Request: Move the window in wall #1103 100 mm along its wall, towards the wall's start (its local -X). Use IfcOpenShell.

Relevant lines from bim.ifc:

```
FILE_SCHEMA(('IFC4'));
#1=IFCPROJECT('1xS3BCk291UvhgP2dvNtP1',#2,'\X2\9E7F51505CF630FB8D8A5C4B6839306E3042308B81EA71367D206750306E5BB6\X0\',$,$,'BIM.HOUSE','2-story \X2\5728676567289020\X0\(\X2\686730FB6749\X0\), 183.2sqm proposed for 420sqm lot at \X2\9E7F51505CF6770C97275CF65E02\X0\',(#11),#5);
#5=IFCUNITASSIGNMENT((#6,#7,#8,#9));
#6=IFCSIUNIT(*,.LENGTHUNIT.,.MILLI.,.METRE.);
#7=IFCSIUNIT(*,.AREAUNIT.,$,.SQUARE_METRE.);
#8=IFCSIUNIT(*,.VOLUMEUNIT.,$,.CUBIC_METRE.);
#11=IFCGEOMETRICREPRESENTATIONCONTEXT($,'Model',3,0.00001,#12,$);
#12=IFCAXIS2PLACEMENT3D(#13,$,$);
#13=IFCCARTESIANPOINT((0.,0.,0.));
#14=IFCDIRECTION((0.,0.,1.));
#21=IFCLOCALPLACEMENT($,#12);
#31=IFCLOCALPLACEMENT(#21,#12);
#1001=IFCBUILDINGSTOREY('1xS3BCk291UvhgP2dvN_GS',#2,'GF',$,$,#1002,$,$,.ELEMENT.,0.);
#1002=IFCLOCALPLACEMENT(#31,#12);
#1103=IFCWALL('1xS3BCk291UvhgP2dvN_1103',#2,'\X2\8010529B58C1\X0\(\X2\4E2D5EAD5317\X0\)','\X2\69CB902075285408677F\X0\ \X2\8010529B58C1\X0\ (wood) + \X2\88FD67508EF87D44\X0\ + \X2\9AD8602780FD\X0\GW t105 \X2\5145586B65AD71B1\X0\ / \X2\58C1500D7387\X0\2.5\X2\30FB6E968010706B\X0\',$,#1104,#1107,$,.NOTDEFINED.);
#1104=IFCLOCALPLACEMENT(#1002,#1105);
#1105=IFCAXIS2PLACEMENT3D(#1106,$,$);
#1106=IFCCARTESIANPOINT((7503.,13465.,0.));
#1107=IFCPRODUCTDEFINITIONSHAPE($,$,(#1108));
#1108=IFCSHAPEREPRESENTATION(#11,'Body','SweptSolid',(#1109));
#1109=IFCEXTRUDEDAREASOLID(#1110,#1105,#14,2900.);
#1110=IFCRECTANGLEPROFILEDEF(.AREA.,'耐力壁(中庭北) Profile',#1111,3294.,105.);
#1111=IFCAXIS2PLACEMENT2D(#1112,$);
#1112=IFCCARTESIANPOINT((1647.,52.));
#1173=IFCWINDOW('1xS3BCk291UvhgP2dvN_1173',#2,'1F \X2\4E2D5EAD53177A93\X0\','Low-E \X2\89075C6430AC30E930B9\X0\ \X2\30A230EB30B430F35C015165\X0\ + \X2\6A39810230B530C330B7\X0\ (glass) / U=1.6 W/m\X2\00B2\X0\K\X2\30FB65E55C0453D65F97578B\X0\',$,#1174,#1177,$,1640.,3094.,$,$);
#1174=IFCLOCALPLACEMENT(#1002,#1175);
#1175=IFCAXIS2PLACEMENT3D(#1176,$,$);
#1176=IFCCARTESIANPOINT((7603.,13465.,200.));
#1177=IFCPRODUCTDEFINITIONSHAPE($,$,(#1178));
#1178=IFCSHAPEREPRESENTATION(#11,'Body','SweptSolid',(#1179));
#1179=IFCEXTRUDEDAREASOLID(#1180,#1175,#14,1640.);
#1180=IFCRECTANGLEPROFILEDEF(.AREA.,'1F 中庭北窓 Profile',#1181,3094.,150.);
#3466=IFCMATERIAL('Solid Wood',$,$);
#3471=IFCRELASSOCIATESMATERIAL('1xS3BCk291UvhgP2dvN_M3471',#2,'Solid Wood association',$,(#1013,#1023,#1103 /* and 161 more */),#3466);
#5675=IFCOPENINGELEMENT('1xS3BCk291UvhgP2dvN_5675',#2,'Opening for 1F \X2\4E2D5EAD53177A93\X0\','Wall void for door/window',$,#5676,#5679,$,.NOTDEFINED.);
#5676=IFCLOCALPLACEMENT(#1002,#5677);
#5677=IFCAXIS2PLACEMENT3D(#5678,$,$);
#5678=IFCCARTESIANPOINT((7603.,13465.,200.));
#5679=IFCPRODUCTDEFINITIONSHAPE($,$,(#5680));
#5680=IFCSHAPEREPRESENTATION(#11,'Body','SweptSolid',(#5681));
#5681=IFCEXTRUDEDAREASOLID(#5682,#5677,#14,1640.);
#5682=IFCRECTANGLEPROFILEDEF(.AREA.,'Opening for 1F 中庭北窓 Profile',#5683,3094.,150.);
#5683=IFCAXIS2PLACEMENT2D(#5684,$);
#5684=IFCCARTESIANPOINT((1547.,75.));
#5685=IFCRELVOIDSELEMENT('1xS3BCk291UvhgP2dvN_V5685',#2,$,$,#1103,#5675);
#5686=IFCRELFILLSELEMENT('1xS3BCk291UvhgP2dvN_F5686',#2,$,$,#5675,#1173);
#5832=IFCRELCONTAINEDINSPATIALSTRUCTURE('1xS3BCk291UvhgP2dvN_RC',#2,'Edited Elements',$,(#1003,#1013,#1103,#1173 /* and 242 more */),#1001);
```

```python
import ifcopenshell
import ifcopenshell.api.geometry
import ifcopenshell.util.placement
import ifcopenshell.util.unit

model = ifcopenshell.open("bim.ifc")
unit_scale = ifcopenshell.util.unit.calculate_unit_scale(model)

window = model.by_guid("1xS3BCk291UvhgP2dvN_1173")
opening = window.FillsVoids[0].RelatingOpeningElement
wall = opening.VoidsElements[0].RelatingBuildingElement

wall_matrix = ifcopenshell.util.placement.get_local_placement(wall.ObjectPlacement)
shift = wall_matrix[:3, 0] * -0.1 / unit_scale
before = ifcopenshell.util.placement.get_local_placement(window.ObjectPlacement)[:3, 3].copy()

# The window is not placed relative to its opening, so move both.
for product in (opening, window):
    matrix = ifcopenshell.util.placement.get_local_placement(product.ObjectPlacement)
    matrix[:3, 3] += shift
    ifcopenshell.api.geometry.edit_object_placement(model, product=product, matrix=matrix, is_si=False)

after = ifcopenshell.util.placement.get_local_placement(window.ObjectPlacement)[:3, 3]
print("window moved by", (after - before).round(3) + 0.0)

model.write("bim_edited.ifc")
```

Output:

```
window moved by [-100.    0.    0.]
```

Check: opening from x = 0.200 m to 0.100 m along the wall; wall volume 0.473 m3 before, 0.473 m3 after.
